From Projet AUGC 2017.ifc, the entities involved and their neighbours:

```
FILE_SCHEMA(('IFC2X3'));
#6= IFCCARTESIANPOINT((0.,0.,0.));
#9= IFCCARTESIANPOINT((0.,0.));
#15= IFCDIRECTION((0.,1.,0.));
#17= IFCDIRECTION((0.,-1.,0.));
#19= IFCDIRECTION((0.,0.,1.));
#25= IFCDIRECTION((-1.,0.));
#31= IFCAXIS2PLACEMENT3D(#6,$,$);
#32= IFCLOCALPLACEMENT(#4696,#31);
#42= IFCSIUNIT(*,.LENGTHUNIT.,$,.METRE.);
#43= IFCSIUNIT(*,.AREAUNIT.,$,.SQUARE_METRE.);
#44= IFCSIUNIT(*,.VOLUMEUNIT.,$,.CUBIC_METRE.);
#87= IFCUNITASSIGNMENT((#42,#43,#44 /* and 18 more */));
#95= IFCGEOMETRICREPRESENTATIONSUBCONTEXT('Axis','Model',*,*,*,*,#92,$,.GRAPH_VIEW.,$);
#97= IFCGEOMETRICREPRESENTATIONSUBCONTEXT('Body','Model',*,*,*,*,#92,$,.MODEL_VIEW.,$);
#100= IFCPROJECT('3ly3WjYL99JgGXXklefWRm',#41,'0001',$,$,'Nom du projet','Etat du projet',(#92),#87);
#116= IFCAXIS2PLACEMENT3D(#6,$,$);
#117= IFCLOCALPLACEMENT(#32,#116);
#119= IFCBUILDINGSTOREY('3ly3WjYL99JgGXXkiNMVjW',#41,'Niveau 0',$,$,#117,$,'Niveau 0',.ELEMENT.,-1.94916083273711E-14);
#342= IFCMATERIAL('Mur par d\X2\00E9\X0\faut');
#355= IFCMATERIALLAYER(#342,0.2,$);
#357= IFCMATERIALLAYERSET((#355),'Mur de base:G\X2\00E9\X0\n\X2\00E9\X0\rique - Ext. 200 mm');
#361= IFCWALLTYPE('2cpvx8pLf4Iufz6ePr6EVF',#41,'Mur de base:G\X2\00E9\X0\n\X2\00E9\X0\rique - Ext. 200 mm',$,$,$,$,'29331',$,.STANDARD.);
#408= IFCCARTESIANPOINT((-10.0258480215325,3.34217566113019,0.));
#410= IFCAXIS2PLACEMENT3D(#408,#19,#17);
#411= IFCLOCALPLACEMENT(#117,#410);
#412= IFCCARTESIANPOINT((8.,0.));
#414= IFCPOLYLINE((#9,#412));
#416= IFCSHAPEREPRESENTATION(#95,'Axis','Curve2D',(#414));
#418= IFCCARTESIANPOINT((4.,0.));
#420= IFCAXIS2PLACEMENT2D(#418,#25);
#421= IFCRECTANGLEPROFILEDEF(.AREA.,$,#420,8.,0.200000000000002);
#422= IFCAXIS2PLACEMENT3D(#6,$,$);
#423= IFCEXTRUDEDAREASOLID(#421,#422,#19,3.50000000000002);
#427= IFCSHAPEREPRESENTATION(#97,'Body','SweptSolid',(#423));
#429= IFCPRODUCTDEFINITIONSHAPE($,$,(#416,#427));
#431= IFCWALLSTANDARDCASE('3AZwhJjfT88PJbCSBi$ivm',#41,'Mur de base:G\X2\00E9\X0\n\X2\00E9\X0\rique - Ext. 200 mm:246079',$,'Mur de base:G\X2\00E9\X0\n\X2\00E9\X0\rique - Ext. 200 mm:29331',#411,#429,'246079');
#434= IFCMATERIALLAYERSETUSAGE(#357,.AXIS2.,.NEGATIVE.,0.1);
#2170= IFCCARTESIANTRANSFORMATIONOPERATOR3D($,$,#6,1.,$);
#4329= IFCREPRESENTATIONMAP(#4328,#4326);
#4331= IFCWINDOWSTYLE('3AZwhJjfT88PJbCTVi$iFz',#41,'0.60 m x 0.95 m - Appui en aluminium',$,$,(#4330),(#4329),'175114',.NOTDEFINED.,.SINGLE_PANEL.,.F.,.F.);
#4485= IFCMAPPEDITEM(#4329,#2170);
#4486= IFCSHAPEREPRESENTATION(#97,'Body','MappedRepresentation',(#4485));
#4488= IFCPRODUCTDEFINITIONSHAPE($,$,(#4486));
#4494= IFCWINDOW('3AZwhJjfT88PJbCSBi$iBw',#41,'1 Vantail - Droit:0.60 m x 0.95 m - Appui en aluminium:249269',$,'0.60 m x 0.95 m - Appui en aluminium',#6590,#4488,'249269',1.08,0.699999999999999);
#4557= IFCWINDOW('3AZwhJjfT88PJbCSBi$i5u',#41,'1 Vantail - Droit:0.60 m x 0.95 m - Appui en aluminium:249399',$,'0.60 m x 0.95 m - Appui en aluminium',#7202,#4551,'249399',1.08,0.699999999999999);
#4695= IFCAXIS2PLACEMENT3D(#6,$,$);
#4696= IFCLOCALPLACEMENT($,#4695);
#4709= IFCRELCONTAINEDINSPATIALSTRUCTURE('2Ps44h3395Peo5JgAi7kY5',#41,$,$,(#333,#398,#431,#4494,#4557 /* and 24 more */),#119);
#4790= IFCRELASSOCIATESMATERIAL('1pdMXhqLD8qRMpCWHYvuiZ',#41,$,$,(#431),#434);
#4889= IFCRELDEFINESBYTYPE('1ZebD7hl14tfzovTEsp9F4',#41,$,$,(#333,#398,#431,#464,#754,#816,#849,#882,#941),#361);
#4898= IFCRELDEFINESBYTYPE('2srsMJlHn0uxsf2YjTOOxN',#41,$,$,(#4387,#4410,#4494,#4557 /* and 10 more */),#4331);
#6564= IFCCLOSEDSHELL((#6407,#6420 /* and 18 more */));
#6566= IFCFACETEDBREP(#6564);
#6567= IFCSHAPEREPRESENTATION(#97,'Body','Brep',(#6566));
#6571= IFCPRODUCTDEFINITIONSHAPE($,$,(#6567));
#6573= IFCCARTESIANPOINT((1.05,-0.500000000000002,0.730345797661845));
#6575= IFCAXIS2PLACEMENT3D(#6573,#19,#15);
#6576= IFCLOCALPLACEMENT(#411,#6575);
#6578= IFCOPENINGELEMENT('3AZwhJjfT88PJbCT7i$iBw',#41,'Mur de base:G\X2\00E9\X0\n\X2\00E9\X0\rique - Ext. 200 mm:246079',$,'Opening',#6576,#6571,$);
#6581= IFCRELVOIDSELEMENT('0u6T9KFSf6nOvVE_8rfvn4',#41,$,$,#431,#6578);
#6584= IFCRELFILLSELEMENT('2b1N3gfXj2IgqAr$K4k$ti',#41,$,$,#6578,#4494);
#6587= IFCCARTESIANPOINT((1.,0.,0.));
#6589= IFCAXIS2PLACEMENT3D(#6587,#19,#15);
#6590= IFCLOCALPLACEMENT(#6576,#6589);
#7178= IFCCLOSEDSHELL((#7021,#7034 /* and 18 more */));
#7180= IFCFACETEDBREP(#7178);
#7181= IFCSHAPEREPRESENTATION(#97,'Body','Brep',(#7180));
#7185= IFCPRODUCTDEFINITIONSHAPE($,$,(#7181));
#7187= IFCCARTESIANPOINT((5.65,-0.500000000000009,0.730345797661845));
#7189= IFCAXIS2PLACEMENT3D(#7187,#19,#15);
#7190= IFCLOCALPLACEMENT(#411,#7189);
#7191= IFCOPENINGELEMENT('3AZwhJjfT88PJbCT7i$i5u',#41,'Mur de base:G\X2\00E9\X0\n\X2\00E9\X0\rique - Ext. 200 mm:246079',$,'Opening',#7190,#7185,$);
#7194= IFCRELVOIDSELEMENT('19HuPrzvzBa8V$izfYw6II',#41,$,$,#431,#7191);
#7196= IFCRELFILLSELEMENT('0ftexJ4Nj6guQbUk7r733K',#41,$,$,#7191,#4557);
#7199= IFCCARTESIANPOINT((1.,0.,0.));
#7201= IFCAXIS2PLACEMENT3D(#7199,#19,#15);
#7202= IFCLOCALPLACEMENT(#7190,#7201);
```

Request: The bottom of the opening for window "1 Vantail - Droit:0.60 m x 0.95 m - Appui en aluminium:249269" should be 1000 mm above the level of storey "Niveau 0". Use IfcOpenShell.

```python
import numpy as np
import ifcopenshell
import ifcopenshell.api.geometry
import ifcopenshell.geom
import ifcopenshell.util.element
import ifcopenshell.util.placement
import ifcopenshell.util.shape
import ifcopenshell.util.unit

model = ifcopenshell.open("Projet AUGC 2017.ifc")
unit_scale = ifcopenshell.util.unit.calculate_unit_scale(model)

window = model.by_guid("3AZwhJjfT88PJbCSBi$iBw")
opening = window.FillsVoids[0].RelatingOpeningElement
storey = ifcopenshell.util.element.get_container(window, ifc_class="IfcBuildingStorey")
level = ifcopenshell.util.placement.get_local_placement(storey.ObjectPlacement)[2, 3]

# The opening's origin need not be at the sill, so measure its lowest point.
shape = ifcopenshell.geom.create_shape(ifcopenshell.geom.settings(), opening)
bottom = ifcopenshell.util.shape.get_shape_bottom_elevation(shape, shape.geometry) / unit_scale
dz = level + 1 / unit_scale - bottom

shift = np.array([0.0, 0.0, dz])
# The window is placed relative to its opening, so it follows when the opening moves.
matrix = ifcopenshell.util.placement.get_local_placement(opening.ObjectPlacement)
matrix[:3, 3] += shift
ifcopenshell.api.geometry.edit_object_placement(
    model, product=opening, matrix=matrix, is_si=False, should_transform_children=True
)

print(f"moved by {dz * unit_scale:+.3f} m")

model.write("Projet AUGC 2017_v2.ifc")
```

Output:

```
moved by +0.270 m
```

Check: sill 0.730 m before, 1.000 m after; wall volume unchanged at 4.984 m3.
